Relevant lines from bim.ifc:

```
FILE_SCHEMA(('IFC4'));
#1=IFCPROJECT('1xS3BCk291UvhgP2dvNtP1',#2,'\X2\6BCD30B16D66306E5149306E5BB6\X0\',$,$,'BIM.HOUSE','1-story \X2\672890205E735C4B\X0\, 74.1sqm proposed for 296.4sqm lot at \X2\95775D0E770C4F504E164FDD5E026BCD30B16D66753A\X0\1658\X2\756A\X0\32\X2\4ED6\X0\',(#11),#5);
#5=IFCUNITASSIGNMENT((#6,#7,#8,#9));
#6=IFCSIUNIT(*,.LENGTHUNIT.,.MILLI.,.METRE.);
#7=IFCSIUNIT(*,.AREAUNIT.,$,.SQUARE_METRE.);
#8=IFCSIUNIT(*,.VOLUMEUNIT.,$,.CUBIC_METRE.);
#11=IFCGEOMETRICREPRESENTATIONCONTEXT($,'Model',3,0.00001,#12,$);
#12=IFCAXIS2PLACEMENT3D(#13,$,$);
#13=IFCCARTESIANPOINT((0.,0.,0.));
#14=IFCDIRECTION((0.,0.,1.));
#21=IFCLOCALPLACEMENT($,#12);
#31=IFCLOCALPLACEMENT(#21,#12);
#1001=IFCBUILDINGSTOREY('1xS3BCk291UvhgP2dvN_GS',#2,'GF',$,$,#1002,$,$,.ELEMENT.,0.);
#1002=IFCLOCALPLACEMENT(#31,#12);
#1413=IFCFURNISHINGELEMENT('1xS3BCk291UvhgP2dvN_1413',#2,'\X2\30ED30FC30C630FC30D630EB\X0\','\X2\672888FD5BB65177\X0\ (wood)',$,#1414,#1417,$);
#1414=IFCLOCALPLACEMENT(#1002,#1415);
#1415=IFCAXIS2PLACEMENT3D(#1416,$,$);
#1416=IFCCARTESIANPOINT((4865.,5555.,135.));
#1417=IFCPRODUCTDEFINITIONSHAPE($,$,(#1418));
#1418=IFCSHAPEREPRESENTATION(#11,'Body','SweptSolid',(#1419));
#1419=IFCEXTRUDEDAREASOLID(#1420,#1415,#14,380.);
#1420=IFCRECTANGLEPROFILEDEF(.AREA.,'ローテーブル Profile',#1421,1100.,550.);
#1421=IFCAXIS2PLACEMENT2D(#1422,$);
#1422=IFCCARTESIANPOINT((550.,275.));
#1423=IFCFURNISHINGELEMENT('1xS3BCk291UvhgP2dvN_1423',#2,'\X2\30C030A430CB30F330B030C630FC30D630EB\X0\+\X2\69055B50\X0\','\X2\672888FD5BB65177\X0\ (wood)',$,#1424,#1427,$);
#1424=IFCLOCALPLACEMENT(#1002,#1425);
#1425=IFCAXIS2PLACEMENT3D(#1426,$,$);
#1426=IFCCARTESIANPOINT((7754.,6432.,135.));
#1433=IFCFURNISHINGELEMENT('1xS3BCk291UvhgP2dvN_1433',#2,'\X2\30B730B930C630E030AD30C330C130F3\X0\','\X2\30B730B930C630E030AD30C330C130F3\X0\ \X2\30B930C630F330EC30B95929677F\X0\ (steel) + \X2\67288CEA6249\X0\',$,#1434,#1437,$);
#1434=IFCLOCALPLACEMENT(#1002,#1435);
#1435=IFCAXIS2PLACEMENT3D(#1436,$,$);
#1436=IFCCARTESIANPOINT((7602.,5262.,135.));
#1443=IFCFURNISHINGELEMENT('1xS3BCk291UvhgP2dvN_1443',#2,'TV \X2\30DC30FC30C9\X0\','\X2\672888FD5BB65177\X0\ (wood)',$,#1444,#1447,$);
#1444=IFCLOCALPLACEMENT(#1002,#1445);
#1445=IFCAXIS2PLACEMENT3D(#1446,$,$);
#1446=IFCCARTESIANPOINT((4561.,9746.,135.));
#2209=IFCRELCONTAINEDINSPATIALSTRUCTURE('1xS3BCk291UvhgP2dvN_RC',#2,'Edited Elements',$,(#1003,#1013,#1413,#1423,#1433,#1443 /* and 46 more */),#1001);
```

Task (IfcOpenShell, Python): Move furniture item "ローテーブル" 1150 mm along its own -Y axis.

```python
import ifcopenshell
import ifcopenshell.api.geometry
import ifcopenshell.util.placement
import ifcopenshell.util.unit

model = ifcopenshell.open("bim.ifc")
unit_scale = ifcopenshell.util.unit.calculate_unit_scale(model)

item = model.by_guid("1xS3BCk291UvhgP2dvN_1413")
matrix = ifcopenshell.util.placement.get_local_placement(item.ObjectPlacement)
matrix[:3, 3] -= matrix[:3, 1] * 1.15 / unit_scale
ifcopenshell.api.geometry.edit_object_placement(model, product=item, matrix=matrix, is_si=False)

print(ifcopenshell.util.placement.get_local_placement(item.ObjectPlacement).round(3) + 0.0)

model.write("bim-out.ifc")
```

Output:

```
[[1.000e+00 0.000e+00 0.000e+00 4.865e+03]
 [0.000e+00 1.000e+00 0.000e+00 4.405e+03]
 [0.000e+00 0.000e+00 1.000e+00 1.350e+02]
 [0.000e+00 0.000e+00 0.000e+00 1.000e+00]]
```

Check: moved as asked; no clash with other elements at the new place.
